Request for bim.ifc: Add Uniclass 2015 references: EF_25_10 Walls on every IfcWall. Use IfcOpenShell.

First a look at what the model holds.

```python
import ifcopenshell

model = ifcopenshell.open("bim.ifc")
print(model.schema)
print("classifications:", [c.Name for c in model.by_type("IfcClassification")])
for ifc_class in ("IfcDoor", "IfcRoof", "IfcStair", "IfcWall", "IfcWindow"):
    print(ifc_class, len(model.by_type(ifc_class)))
```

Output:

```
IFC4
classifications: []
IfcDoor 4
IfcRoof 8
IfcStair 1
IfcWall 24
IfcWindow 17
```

```python
import ifcopenshell
import ifcopenshell.api.classification

model = ifcopenshell.open("bim.ifc")

system = ifcopenshell.api.classification.add_classification(model, classification="Uniclass 2015")

codes = {
    "IfcWall": ("EF_25_10", "Walls"),
}
for ifc_class, (code, name) in codes.items():
    products = model.by_type(ifc_class)
    ifcopenshell.api.classification.add_reference(
        model, products=products, classification=system, identification=code, name=name
    )
    print(code, len(products))

model.write("bim_rev.ifc")
```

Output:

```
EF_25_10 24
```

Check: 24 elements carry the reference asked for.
